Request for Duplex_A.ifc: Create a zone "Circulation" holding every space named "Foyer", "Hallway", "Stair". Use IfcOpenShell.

First a look at what the model holds.

```python
import ifcopenshell

model = ifcopenshell.open("Duplex_A.ifc")
print(model.schema)
seen = {}
for space in model.by_type("IfcSpace"):
    seen[space.LongName] = seen.get(space.LongName, 0) + 1
for name, count in sorted(seen.items(), key=str):
    print(count, "x", name)
print("zones:", [z.Name for z in model.by_type("IfcZone")][:20])
```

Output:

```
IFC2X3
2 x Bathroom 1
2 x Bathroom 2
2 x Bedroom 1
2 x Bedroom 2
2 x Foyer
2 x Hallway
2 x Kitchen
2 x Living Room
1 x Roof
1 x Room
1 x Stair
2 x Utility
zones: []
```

```python
import ifcopenshell
import ifcopenshell.api.group
import ifcopenshell.api.root

model = ifcopenshell.open("Duplex_A.ifc")

names = {"Foyer", "Hallway", "Stair"}
spaces = [s for s in model.by_type("IfcSpace") if s.LongName in names]

zone = ifcopenshell.api.root.create_entity(model, ifc_class="IfcZone", name="Circulation")
ifcopenshell.api.group.assign_group(model, products=spaces, group=zone)
print(len(spaces), "spaces in", zone.Name)

model.write("Duplex_A_v2.ifc")
```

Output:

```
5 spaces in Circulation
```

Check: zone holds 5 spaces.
